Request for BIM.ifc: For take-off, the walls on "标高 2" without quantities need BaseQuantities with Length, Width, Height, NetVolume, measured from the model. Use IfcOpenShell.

First a look at what the model holds.

```python
import ifcopenshell
import ifcopenshell.util.element
import ifcopenshell.util.unit

model = ifcopenshell.open("BIM.ifc")
print(model.schema)
for unit_type in ("LENGTHUNIT", "AREAUNIT", "VOLUMEUNIT"):
    print(unit_type, ifcopenshell.util.unit.calculate_unit_scale(model, unit_type))
storey = next(s for s in model.by_type("IfcBuildingStorey") if s.Name == "标高 2")
walls = [e for e in ifcopenshell.util.element.get_decomposition(storey) if e.is_a("IfcWall")]
for e in sorted(walls, key=lambda e: e.id()):
    print(e.id(), e.is_a(), e.Name, list(ifcopenshell.util.element.get_psets(e, qtos_only=True)), sep=" | ")
```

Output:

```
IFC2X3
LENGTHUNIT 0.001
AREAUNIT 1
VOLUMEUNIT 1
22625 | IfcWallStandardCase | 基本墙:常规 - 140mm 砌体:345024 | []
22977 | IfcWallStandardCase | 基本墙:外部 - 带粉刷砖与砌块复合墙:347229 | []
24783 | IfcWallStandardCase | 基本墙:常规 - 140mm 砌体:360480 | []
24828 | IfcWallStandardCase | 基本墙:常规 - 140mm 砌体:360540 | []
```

```python
import ifcopenshell
import ifcopenshell.api.pset
import ifcopenshell.geom
import ifcopenshell.util.element
import ifcopenshell.util.shape
import ifcopenshell.util.unit

model = ifcopenshell.open("BIM.ifc")
unit_scale = ifcopenshell.util.unit.calculate_unit_scale(model)
volume_scale = ifcopenshell.util.unit.calculate_unit_scale(model, "VOLUMEUNIT")
settings = ifcopenshell.geom.settings()

storey = next(s for s in model.by_type("IfcBuildingStorey") if s.Name == "标高 2")
walls = [e for e in ifcopenshell.util.element.get_decomposition(storey) if e.is_a("IfcWall")]

for e in sorted(walls, key=lambda e: e.id()):
    if ifcopenshell.util.element.get_psets(e, qtos_only=True, should_inherit=False):
        continue
    # Geometry comes back in metres, in the element's own axes.
    shape = ifcopenshell.geom.create_shape(settings, e)
    values = {
        "Length": ifcopenshell.util.shape.get_x(shape.geometry) / unit_scale,
        "Width": ifcopenshell.util.shape.get_y(shape.geometry) / unit_scale,
        "Height": ifcopenshell.util.shape.get_z(shape.geometry) / unit_scale,
        "NetVolume": ifcopenshell.util.shape.get_volume(shape.geometry) / volume_scale,
    }
    qto = ifcopenshell.api.pset.add_qto(model, product=e, name="BaseQuantities")
    ifcopenshell.api.pset.edit_qto(model, qto=qto, properties=values)
    print(e.id(), {k: round(v, 3) for k, v in values.items()})

model.write("BIM-out.ifc")
```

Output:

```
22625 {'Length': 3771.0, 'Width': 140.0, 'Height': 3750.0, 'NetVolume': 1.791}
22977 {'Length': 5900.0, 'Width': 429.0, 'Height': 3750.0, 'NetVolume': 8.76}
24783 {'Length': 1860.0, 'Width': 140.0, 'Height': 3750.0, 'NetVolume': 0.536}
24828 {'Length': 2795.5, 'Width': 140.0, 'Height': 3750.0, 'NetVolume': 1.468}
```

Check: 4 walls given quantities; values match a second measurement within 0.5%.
